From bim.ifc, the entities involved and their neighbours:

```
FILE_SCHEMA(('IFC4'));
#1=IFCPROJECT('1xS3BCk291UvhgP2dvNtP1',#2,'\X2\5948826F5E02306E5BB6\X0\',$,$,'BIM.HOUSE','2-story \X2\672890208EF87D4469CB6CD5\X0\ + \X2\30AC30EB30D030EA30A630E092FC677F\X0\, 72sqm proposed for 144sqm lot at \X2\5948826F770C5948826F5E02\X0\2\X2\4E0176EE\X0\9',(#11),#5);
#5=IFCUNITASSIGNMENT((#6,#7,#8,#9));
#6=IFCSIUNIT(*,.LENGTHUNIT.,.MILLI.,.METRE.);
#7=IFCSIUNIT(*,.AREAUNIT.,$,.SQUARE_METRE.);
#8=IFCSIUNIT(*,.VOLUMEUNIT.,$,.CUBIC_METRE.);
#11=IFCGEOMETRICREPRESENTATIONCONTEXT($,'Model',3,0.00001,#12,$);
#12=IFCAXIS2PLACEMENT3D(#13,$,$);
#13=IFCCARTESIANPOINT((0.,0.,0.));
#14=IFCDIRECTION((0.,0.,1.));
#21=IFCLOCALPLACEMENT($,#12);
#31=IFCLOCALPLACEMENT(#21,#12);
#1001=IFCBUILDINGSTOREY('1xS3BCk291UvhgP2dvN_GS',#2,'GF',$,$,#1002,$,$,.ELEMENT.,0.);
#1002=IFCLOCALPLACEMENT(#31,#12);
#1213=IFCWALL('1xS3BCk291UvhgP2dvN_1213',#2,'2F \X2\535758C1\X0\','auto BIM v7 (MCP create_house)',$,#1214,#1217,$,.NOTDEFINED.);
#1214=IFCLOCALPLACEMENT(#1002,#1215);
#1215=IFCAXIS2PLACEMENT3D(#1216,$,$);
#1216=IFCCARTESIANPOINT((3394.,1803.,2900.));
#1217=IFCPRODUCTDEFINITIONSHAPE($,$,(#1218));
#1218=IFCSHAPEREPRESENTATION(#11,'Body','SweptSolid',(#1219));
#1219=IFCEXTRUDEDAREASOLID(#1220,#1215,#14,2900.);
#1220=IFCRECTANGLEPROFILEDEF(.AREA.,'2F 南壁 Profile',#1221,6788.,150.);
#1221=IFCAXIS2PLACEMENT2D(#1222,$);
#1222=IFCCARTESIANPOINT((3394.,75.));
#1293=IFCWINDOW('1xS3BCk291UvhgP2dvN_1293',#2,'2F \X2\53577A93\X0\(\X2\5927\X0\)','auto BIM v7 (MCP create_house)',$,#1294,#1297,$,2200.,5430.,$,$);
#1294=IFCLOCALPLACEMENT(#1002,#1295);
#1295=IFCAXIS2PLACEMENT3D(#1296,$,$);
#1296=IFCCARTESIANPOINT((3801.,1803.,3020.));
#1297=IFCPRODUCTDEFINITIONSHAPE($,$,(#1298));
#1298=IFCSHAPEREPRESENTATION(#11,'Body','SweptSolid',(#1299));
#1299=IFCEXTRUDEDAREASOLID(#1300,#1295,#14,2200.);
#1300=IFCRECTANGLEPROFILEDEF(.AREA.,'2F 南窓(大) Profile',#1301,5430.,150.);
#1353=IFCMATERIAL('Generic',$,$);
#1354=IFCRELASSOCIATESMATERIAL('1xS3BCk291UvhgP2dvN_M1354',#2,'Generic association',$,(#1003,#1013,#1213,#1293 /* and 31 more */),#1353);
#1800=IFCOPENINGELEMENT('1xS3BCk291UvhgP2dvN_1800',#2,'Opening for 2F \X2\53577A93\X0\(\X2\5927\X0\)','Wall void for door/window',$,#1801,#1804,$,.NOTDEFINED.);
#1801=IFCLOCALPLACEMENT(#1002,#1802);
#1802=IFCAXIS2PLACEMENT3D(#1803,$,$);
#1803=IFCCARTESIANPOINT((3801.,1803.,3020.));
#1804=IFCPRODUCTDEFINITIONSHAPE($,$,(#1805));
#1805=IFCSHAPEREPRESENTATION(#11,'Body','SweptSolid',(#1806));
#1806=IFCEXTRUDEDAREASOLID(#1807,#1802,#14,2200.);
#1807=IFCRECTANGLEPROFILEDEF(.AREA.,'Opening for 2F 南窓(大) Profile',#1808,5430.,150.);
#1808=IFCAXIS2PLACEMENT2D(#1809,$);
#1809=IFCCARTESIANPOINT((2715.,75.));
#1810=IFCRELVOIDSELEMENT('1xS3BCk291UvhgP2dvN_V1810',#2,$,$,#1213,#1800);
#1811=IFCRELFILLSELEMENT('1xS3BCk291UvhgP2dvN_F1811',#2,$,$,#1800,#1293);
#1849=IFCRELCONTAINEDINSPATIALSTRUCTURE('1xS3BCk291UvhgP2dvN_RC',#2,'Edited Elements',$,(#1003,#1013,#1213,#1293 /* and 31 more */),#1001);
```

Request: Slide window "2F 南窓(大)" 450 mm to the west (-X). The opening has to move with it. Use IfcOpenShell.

```python
import ifcopenshell
import ifcopenshell.api.geometry
import ifcopenshell.util.placement
import ifcopenshell.util.unit

model = ifcopenshell.open("bim.ifc")
unit_scale = ifcopenshell.util.unit.calculate_unit_scale(model)

window = model.by_guid("1xS3BCk291UvhgP2dvN_1293")
opening = window.FillsVoids[0].RelatingOpeningElement
wall = opening.VoidsElements[0].RelatingBuildingElement

wall_matrix = ifcopenshell.util.placement.get_local_placement(wall.ObjectPlacement)
shift = wall_matrix[:3, 0] * -0.45 / unit_scale
before = ifcopenshell.util.placement.get_local_placement(window.ObjectPlacement)[:3, 3].copy()

# The window is not placed relative to its opening, so move both.
for product in (opening, window):
    matrix = ifcopenshell.util.placement.get_local_placement(product.ObjectPlacement)
    matrix[:3, 3] += shift
    ifcopenshell.api.geometry.edit_object_placement(model, product=product, matrix=matrix, is_si=False)

after = ifcopenshell.util.placement.get_local_placement(window.ObjectPlacement)[:3, 3]
print("window moved by", (after - before).round(3) + 0.0)

model.write("bim-out.ifc")
```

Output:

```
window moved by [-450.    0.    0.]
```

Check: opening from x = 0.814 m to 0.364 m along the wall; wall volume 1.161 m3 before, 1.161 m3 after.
